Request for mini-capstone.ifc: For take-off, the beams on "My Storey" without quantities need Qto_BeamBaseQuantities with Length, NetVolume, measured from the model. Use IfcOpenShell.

First a look at what the model holds.

```python
import ifcopenshell
import ifcopenshell.util.element
import ifcopenshell.util.unit

model = ifcopenshell.open("mini-capstone.ifc")
print(model.schema)
for unit_type in ("LENGTHUNIT", "AREAUNIT", "VOLUMEUNIT"):
    print(unit_type, ifcopenshell.util.unit.calculate_unit_scale(model, unit_type))
storey = next(s for s in model.by_type("IfcBuildingStorey") if s.Name == "My Storey")
beams = [e for e in ifcopenshell.util.element.get_decomposition(storey) if e.is_a("IfcBeam")]
for e in sorted(beams, key=lambda e: e.id()):
    print(e.id(), e.is_a(), e.Name, list(ifcopenshell.util.element.get_psets(e, qtos_only=True)), sep=" | ")
```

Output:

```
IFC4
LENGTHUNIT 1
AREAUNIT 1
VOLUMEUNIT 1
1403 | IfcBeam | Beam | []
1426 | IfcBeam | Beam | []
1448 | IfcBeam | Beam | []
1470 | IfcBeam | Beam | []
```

```python
import ifcopenshell
import ifcopenshell.api.pset
import ifcopenshell.geom
import ifcopenshell.util.element
import ifcopenshell.util.shape
import ifcopenshell.util.unit

model = ifcopenshell.open("mini-capstone.ifc")
unit_scale = ifcopenshell.util.unit.calculate_unit_scale(model)
volume_scale = ifcopenshell.util.unit.calculate_unit_scale(model, "VOLUMEUNIT")
settings = ifcopenshell.geom.settings()

storey = next(s for s in model.by_type("IfcBuildingStorey") if s.Name == "My Storey")
beams = [e for e in ifcopenshell.util.element.get_decomposition(storey) if e.is_a("IfcBeam")]

for e in sorted(beams, key=lambda e: e.id()):
    if ifcopenshell.util.element.get_psets(e, qtos_only=True, should_inherit=False):
        continue
    # Geometry comes back in metres, in the element's own axes.
    shape = ifcopenshell.geom.create_shape(settings, e)
    values = {
        "Length": ifcopenshell.util.shape.get_max_xyz(shape.geometry) / unit_scale,
        "NetVolume": ifcopenshell.util.shape.get_volume(shape.geometry) / volume_scale,
    }
    qto = ifcopenshell.api.pset.add_qto(model, product=e, name="Qto_BeamBaseQuantities")
    ifcopenshell.api.pset.edit_qto(model, qto=qto, properties=values)
    print(e.id(), {k: round(v, 3) for k, v in values.items()})

model.write("mini-capstone_v2.ifc")
```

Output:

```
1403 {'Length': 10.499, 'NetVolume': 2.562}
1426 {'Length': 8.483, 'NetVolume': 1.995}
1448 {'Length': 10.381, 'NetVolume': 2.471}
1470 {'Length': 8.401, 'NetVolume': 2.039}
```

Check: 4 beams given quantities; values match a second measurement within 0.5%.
